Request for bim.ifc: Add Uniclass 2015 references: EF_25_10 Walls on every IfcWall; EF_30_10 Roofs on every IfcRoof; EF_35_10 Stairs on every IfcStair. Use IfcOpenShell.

First a look at what the model holds.

```python
import ifcopenshell

model = ifcopenshell.open("bim.ifc")
print(model.schema)
print("classifications:", [c.Name for c in model.by_type("IfcClassification")])
for ifc_class in ("IfcDoor", "IfcRoof", "IfcStair", "IfcWall", "IfcWindow"):
    print(ifc_class, len(model.by_type(ifc_class)))
```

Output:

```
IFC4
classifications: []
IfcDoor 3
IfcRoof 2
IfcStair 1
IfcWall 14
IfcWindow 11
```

```python
import ifcopenshell
import ifcopenshell.api.classification

model = ifcopenshell.open("bim.ifc")

system = ifcopenshell.api.classification.add_classification(model, classification="Uniclass 2015")

codes = {
    "IfcWall": ("EF_25_10", "Walls"),
    "IfcRoof": ("EF_30_10", "Roofs"),
    "IfcStair": ("EF_35_10", "Stairs"),
}
for ifc_class, (code, name) in codes.items():
    products = model.by_type(ifc_class)
    ifcopenshell.api.classification.add_reference(
        model, products=products, classification=system, identification=code, name=name
    )
    print(code, len(products))

model.write("bim_v2.ifc")
```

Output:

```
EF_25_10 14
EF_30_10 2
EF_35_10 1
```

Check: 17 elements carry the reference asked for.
